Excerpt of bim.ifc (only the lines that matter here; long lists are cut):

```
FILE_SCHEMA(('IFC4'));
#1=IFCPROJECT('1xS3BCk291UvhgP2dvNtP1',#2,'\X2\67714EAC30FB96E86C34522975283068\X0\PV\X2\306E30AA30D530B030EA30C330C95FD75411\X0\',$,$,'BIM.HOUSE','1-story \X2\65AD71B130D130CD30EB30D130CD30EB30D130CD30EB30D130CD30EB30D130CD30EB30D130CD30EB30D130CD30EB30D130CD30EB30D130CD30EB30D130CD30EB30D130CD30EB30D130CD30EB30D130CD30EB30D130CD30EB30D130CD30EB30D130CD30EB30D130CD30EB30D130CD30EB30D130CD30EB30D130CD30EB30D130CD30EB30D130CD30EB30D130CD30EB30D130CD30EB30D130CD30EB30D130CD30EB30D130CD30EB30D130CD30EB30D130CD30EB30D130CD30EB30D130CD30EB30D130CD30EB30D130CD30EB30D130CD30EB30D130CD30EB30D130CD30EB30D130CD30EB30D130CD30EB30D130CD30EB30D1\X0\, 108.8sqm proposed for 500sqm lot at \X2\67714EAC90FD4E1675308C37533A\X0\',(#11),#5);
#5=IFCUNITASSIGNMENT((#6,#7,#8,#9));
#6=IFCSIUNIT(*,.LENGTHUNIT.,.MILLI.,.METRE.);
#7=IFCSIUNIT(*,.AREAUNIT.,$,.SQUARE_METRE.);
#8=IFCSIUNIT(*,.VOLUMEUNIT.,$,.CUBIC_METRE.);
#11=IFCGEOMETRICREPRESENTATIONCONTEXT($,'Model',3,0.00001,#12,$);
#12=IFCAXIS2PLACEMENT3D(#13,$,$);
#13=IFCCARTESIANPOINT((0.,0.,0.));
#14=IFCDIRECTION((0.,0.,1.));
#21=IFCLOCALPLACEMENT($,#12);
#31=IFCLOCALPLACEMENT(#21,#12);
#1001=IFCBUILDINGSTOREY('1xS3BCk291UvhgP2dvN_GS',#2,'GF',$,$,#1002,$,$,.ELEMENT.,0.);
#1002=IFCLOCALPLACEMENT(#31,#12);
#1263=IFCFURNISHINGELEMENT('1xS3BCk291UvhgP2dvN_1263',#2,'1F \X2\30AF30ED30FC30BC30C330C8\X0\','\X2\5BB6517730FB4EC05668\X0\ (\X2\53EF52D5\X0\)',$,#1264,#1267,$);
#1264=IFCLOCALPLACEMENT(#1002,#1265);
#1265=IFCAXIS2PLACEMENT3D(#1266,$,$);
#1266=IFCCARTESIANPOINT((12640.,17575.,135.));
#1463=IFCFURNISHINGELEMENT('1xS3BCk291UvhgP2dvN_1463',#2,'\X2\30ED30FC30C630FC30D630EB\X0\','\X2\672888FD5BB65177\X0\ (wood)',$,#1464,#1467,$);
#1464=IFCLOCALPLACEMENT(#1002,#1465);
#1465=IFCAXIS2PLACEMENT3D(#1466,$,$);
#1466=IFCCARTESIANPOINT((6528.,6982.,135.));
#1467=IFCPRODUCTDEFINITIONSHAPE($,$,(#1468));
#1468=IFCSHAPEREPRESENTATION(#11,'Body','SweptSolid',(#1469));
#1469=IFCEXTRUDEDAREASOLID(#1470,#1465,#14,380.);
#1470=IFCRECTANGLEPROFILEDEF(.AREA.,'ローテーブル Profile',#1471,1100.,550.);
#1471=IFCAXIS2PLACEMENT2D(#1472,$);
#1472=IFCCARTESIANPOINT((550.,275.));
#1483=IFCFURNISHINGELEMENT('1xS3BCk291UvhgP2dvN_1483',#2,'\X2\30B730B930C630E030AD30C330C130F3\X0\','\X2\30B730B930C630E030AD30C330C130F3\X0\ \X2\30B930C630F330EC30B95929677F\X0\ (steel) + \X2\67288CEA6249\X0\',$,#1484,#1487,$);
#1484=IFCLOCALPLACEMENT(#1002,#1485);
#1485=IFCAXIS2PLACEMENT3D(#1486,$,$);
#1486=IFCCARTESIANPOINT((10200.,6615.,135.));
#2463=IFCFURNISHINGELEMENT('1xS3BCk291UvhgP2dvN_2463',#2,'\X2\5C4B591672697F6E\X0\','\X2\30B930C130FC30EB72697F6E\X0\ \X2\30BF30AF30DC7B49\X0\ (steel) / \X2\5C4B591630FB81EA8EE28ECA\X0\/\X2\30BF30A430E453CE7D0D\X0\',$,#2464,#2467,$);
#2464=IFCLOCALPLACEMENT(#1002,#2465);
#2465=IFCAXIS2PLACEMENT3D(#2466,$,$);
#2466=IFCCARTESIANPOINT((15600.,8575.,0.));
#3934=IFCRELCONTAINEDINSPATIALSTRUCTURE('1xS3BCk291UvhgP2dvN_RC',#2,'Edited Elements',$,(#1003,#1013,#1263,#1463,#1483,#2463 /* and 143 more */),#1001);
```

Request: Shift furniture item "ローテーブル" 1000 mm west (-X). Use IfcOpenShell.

```python
import ifcopenshell
import ifcopenshell.api.geometry
import ifcopenshell.util.placement
import ifcopenshell.util.unit

model = ifcopenshell.open("bim.ifc")
unit_scale = ifcopenshell.util.unit.calculate_unit_scale(model)

item = model.by_guid("1xS3BCk291UvhgP2dvN_1463")
matrix = ifcopenshell.util.placement.get_local_placement(item.ObjectPlacement)
matrix[0, 3] -= 1 / unit_scale
ifcopenshell.api.geometry.edit_object_placement(model, product=item, matrix=matrix, is_si=False)

print(ifcopenshell.util.placement.get_local_placement(item.ObjectPlacement).round(3) + 0.0)

model.write("bim_edited.ifc")
```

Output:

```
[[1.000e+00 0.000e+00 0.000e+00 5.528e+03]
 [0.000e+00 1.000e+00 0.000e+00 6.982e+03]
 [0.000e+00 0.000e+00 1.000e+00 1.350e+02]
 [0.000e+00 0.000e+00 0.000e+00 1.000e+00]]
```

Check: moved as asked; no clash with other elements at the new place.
